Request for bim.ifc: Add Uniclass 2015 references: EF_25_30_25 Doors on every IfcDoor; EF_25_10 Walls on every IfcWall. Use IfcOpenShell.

First a look at what the model holds.

```python
import ifcopenshell

model = ifcopenshell.open("bim.ifc")
print(model.schema)
print("classifications:", [c.Name for c in model.by_type("IfcClassification")])
for ifc_class in ("IfcDoor", "IfcRoof", "IfcStair", "IfcWall", "IfcWindow"):
    print(ifc_class, len(model.by_type(ifc_class)))
```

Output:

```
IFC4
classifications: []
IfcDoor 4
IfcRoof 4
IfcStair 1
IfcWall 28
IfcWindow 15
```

```python
import ifcopenshell
import ifcopenshell.api.classification

model = ifcopenshell.open("bim.ifc")

system = ifcopenshell.api.classification.add_classification(model, classification="Uniclass 2015")

codes = {
    "IfcDoor": ("EF_25_30_25", "Doors"),
    "IfcWall": ("EF_25_10", "Walls"),
}
for ifc_class, (code, name) in codes.items():
    products = model.by_type(ifc_class)
    ifcopenshell.api.classification.add_reference(
        model, products=products, classification=system, identification=code, name=name
    )
    print(code, len(products))

model.write("bim-out.ifc")
```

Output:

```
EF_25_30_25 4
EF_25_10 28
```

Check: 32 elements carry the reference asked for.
